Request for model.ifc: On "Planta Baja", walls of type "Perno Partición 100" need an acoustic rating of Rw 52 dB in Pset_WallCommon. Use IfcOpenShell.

First a look at what the model holds.

```python
import ifcopenshell
import ifcopenshell.util.element

model = ifcopenshell.open("model.ifc")
print(model.schema)
storey = next(s for s in model.by_type("IfcBuildingStorey") if s.Name == "Planta Baja")
walls = [e for e in ifcopenshell.util.element.get_decomposition(storey) if e.is_a("IfcWall")]
seen = {}
for e in walls:
    element_type = ifcopenshell.util.element.get_type(e)
    key = (element_type.Name if element_type != e and element_type else None, ifcopenshell.util.element.get_pset(e, "Pset_WallCommon", "AcousticRating"))
    seen[key] = seen.get(key, 0) + 1
for (name, value), count in sorted(seen.items(), key=str):
    print(count, "x", name, "|", value)
```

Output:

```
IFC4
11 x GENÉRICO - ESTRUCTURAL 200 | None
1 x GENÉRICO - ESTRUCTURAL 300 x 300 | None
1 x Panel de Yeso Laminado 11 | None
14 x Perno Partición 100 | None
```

```python
import ifcopenshell
import ifcopenshell.api.pset
import ifcopenshell.util.element

model = ifcopenshell.open("model.ifc")

storey = next(s for s in model.by_type("IfcBuildingStorey") if s.Name == "Planta Baja")
walls = [e for e in ifcopenshell.util.element.get_decomposition(storey) if e.is_a("IfcWall")]

count = 0
for e in walls:
    element_type = ifcopenshell.util.element.get_type(e)
    if element_type in (None, e) or element_type.Name != "Perno Partición 100":
        continue
    # add_pset returns the element's existing set when there is one.
    pset = ifcopenshell.api.pset.add_pset(model, product=e, name="Pset_WallCommon")
    ifcopenshell.api.pset.edit_pset(model, pset=pset, properties={"AcousticRating": "Rw 52 dB"})
    count += 1

print(count, "walls updated")

model.write("model_updated.ifc")
```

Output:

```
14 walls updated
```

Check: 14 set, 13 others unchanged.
